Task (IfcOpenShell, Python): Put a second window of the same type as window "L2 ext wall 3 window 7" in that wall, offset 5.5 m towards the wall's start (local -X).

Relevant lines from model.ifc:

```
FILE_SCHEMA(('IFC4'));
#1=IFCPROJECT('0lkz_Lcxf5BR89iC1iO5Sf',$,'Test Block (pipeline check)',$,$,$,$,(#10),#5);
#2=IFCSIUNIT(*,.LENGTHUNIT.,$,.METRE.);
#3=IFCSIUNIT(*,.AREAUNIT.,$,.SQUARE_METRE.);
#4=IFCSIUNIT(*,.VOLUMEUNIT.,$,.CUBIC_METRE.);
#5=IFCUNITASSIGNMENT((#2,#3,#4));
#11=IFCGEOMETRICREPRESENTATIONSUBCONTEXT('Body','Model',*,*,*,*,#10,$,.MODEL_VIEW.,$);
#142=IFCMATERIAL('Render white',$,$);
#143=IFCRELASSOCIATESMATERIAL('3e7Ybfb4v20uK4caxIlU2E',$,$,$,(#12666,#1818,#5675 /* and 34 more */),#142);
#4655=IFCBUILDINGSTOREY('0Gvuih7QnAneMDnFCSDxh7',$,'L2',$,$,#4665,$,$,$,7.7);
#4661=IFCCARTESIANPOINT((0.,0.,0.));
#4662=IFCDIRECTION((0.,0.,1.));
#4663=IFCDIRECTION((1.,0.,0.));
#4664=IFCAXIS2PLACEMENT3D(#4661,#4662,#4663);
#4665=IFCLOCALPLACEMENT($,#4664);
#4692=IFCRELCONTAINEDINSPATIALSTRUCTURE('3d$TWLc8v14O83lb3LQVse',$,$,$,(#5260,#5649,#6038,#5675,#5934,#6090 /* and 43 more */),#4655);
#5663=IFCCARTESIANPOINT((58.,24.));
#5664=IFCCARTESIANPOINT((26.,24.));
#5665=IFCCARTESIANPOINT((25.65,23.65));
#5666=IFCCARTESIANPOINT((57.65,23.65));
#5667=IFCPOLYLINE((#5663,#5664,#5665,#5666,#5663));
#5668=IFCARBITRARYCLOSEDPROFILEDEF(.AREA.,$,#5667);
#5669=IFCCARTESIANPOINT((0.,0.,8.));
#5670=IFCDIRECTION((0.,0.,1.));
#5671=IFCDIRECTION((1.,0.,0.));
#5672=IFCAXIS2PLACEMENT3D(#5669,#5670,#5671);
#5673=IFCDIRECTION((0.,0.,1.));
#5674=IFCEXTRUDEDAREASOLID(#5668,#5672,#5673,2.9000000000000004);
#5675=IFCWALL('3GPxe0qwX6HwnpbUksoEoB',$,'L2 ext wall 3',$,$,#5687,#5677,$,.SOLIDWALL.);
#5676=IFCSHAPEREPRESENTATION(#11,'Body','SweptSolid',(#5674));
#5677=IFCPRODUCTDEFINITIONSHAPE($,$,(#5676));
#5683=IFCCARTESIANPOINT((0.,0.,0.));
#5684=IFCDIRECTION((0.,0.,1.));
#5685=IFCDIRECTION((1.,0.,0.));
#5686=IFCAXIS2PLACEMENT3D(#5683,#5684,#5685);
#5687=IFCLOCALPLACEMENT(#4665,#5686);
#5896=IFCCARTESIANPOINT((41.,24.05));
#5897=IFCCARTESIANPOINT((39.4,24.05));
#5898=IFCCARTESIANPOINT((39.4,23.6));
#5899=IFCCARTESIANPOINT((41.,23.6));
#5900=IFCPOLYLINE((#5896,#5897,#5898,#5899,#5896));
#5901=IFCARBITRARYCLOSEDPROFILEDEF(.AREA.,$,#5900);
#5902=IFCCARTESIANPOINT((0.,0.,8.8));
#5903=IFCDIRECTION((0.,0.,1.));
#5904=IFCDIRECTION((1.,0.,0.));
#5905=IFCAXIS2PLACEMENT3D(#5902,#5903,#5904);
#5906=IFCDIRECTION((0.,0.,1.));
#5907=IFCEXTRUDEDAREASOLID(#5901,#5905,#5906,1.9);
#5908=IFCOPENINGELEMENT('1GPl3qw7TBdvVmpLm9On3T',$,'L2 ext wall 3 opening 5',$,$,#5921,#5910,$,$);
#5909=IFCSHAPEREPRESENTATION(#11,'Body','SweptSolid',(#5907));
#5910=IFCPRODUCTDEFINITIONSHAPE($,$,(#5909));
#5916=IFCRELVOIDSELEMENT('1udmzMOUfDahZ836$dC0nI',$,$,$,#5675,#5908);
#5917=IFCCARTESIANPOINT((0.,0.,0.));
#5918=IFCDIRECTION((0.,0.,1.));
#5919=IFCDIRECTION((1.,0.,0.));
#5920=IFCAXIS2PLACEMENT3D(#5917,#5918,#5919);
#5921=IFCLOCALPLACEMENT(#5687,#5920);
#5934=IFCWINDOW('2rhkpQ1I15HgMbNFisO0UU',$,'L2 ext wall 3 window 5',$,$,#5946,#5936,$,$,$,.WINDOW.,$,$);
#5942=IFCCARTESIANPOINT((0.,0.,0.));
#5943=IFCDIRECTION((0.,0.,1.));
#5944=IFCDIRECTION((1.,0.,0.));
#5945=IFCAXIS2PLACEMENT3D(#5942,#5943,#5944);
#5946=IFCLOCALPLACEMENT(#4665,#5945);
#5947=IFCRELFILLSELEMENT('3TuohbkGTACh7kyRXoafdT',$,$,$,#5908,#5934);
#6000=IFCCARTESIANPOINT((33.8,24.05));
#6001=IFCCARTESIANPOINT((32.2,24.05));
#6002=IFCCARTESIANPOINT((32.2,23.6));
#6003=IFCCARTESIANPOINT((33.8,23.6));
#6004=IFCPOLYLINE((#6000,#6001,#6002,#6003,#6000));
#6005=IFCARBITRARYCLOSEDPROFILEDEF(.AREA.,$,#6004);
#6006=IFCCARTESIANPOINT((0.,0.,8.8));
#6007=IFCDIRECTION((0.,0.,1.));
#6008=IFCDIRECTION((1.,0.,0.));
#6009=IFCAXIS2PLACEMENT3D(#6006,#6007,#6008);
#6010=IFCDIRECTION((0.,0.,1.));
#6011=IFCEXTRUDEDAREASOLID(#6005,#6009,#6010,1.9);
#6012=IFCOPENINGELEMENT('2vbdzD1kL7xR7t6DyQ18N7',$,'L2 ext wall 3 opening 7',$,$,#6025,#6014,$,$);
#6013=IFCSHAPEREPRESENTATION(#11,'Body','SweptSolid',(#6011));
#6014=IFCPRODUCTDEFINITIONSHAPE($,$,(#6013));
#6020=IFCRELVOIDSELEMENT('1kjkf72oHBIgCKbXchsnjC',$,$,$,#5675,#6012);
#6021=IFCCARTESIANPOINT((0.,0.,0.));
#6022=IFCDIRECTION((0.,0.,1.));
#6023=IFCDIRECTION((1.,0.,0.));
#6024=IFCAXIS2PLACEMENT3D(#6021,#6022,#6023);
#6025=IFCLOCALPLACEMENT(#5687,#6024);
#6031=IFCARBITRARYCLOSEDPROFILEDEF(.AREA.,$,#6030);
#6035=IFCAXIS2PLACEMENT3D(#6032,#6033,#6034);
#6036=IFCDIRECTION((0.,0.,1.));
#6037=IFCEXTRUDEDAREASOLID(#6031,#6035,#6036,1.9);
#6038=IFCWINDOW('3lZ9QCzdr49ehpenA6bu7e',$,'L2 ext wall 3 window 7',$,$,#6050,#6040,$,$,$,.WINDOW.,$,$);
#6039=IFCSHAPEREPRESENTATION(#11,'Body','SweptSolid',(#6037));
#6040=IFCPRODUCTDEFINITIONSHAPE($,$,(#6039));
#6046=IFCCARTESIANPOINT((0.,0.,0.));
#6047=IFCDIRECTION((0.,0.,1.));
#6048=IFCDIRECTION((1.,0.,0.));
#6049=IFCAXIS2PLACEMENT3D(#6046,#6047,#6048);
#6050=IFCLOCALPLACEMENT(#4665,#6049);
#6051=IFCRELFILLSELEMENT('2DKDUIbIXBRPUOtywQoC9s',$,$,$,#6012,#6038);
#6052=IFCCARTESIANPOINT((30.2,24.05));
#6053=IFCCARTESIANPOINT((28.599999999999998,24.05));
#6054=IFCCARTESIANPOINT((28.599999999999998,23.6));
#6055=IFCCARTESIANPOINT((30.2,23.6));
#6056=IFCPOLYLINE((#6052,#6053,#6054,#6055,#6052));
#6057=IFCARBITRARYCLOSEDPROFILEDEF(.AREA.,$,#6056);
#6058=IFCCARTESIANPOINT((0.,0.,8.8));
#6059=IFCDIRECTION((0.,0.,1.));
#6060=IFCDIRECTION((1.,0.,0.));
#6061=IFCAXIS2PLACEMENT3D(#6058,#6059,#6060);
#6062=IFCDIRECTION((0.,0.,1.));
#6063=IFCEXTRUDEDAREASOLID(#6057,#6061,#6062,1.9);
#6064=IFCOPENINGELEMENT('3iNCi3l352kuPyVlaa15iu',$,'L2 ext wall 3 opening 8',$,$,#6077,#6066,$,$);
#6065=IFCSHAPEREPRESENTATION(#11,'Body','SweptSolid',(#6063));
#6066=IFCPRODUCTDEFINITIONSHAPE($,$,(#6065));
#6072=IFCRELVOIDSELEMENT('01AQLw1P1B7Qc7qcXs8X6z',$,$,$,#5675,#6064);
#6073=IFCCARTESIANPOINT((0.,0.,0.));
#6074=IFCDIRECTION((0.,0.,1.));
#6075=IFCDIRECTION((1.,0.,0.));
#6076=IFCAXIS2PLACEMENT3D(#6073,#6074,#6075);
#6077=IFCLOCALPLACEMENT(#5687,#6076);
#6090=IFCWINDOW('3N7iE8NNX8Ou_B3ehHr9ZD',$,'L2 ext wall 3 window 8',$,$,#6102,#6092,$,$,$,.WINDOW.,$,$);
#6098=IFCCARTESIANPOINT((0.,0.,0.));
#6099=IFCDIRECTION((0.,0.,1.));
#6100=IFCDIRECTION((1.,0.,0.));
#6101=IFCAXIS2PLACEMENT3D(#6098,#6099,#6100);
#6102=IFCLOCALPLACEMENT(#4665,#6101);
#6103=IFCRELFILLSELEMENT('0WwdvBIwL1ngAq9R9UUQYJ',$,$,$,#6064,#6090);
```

```python
import ifcopenshell
import ifcopenshell.api.feature
import ifcopenshell.api.geometry
import ifcopenshell.api.root
import ifcopenshell.geom
import ifcopenshell.util.element
import ifcopenshell.util.placement
import ifcopenshell.util.shape
import ifcopenshell.util.unit

model = ifcopenshell.open("model.ifc")
unit_scale = ifcopenshell.util.unit.calculate_unit_scale(model)
settings = ifcopenshell.geom.settings()


def volume(element):
    """Net volume in cubic metres, openings subtracted."""
    shape = ifcopenshell.geom.create_shape(settings, element)
    return ifcopenshell.util.shape.get_volume(shape.geometry)


window = model.by_guid("3lZ9QCzdr49ehpenA6bu7e")
opening = window.FillsVoids[0].RelatingOpeningElement
wall = opening.VoidsElements[0].RelatingBuildingElement
before = volume(wall)
shift = ifcopenshell.util.placement.get_local_placement(wall.ObjectPlacement)[:3, 0] * -5.5 / unit_scale

# copy_class copies the void relationship, type, container and properties, but no geometry.
new_opening = ifcopenshell.api.root.copy_class(model, product=opening)
new_opening.Representation = ifcopenshell.util.element.copy_deep(
    model, opening.Representation, exclude=["IfcGeometricRepresentationContext", "IfcRepresentationMap"]
)
new_window = ifcopenshell.api.root.copy_class(model, product=window)
new_window.Representation = ifcopenshell.util.element.copy_deep(
    model, window.Representation, exclude=["IfcGeometricRepresentationContext", "IfcRepresentationMap"]
)
ifcopenshell.api.feature.add_filling(model, opening=new_opening, element=new_window)

for old, new in ((opening, new_opening), (window, new_window)):
    matrix = ifcopenshell.util.placement.get_local_placement(old.ObjectPlacement)
    matrix[:3, 3] += shift
    ifcopenshell.api.geometry.edit_object_placement(model, product=new, matrix=matrix, is_si=False)

after = volume(wall)

print(f"wall volume {before:.3f} -> {after:.3f} m3")

model.write("model_v2.ifc")
```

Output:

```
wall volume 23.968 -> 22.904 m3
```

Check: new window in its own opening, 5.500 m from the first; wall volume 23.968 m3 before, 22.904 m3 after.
